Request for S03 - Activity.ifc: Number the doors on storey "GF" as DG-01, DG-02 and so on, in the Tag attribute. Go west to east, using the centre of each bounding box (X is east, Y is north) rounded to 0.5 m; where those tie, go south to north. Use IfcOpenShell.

First a look at what the model holds.

```python
import ifcopenshell
import ifcopenshell.util.element
import ifcopenshell.util.placement

model = ifcopenshell.open("S03 - Activity.ifc")
print(model.schema)
storey = next(s for s in model.by_type("IfcBuildingStorey") if s.Name == "GF")
doors = [e for e in ifcopenshell.util.element.get_decomposition(storey) if e.is_a("IfcDoor")]
for e in sorted(doors, key=lambda e: e.id()):
    origin = ifcopenshell.util.placement.get_local_placement(e.ObjectPlacement)[:3, 3]
    print(e.id(), e.Tag, e.Name, origin.round(2) + 0.0, sep=" | ")
```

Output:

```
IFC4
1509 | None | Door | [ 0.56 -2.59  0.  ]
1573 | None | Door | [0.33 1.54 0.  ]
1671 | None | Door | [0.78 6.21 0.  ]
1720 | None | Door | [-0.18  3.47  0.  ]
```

```python
import ifcopenshell
import ifcopenshell.geom
import ifcopenshell.util.element
import ifcopenshell.util.shape

model = ifcopenshell.open("S03 - Activity.ifc")
settings = ifcopenshell.geom.settings()
settings.set("use-world-coords", True)


def centre(element):
    shape = ifcopenshell.geom.create_shape(settings, element)
    return ifcopenshell.util.shape.get_bbox_centroid(shape.geometry)


storey = next(s for s in model.by_type("IfcBuildingStorey") if s.Name == "GF")
doors = [e for e in ifcopenshell.util.element.get_decomposition(storey) if e.is_a("IfcDoor")]

# Insertion points can sit at a corner or the storey origin, so sort by the geometry (in metres).
centres = {e: centre(e) for e in doors}
doors.sort(key=lambda e: (round(centres[e][0] / 0.5), centres[e][1]))

for i, e in enumerate(doors, start=1):
    number = f"DG-{i:02d}"
    e.Tag = number
    print(e.id(), number)

model.write("S03 - Activity_updated.ifc")
```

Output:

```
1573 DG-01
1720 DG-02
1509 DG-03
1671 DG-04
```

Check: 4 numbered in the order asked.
